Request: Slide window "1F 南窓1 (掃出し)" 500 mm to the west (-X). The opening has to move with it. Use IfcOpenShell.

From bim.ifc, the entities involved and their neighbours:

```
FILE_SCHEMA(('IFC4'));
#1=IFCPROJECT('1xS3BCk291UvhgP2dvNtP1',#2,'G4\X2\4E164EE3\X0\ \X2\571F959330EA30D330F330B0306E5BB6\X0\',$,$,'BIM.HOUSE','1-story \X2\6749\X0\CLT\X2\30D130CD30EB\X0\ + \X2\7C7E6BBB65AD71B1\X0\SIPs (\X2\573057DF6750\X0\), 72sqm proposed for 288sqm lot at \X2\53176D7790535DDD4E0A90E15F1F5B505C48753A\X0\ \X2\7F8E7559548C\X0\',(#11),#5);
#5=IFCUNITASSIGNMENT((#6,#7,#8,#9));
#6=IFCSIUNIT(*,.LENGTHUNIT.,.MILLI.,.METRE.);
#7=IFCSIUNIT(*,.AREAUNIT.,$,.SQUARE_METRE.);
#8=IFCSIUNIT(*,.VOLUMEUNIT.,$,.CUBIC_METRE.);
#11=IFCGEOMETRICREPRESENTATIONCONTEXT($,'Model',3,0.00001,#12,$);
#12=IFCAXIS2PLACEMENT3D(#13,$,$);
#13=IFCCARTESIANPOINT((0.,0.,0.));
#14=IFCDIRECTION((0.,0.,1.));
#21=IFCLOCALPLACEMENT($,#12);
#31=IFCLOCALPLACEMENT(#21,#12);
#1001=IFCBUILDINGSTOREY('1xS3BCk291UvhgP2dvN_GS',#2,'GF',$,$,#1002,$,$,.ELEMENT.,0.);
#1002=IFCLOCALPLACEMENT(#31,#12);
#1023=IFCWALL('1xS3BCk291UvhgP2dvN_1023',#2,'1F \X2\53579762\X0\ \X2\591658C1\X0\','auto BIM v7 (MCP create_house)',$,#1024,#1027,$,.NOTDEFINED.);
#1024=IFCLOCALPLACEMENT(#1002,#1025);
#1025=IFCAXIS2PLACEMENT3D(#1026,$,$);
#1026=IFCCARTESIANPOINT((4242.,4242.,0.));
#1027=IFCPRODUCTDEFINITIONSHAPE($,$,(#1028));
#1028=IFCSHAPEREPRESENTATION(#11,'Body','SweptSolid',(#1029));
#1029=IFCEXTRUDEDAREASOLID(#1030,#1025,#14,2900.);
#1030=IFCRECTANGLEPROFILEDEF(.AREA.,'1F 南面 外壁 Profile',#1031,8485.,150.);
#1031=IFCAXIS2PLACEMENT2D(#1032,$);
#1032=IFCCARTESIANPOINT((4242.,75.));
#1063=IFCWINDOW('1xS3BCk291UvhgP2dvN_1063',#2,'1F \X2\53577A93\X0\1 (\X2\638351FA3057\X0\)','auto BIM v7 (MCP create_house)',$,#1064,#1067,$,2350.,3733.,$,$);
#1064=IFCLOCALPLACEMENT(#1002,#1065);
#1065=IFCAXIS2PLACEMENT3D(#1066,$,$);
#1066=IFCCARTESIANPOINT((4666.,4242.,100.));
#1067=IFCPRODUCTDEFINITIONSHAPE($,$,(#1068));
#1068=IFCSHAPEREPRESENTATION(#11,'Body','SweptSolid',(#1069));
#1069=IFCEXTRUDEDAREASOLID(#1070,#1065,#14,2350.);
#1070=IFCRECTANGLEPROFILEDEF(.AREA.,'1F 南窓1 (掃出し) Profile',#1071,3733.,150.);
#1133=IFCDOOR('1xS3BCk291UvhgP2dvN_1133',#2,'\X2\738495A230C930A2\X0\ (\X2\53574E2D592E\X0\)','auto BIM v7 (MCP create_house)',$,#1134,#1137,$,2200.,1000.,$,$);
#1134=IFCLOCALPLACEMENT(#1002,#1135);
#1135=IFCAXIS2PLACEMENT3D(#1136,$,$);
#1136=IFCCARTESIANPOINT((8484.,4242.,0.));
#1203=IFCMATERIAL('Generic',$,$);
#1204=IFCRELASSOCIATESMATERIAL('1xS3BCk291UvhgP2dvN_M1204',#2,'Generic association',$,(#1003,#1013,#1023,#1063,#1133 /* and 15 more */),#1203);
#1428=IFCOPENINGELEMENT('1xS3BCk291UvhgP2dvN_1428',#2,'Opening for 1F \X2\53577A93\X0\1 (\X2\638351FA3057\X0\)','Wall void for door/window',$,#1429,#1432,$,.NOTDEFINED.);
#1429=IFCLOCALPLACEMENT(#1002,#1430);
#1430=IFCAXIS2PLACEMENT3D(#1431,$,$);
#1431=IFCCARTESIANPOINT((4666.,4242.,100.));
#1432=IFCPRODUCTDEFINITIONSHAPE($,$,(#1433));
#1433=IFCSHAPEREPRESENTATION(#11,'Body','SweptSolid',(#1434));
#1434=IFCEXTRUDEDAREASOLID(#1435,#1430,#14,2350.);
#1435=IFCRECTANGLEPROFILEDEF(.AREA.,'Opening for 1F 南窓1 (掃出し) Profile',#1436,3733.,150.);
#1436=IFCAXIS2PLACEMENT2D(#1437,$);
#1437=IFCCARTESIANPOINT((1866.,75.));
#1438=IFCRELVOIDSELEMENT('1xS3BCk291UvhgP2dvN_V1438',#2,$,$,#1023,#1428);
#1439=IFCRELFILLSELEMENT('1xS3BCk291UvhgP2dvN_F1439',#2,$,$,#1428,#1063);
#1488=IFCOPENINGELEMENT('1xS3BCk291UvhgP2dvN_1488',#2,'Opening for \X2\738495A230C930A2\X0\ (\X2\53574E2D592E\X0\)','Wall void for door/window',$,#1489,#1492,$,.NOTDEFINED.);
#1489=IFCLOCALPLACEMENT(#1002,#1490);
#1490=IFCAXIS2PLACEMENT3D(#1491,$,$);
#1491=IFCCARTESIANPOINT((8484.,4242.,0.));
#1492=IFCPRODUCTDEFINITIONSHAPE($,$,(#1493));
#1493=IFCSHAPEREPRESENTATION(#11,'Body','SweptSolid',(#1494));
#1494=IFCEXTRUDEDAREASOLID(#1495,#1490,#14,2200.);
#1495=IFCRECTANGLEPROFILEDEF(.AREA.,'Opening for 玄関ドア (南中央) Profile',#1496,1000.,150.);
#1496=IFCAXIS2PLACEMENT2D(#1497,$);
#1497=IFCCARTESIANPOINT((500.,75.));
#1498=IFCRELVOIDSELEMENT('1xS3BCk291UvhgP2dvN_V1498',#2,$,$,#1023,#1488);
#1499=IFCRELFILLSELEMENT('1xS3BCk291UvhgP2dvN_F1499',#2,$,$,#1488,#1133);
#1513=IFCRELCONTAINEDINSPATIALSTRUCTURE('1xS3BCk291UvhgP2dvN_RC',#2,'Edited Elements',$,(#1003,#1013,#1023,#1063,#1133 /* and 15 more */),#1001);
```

```python
import ifcopenshell
import ifcopenshell.api.geometry
import ifcopenshell.util.placement
import ifcopenshell.util.unit

model = ifcopenshell.open("bim.ifc")
unit_scale = ifcopenshell.util.unit.calculate_unit_scale(model)

window = model.by_guid("1xS3BCk291UvhgP2dvN_1063")
opening = window.FillsVoids[0].RelatingOpeningElement
wall = opening.VoidsElements[0].RelatingBuildingElement

wall_matrix = ifcopenshell.util.placement.get_local_placement(wall.ObjectPlacement)
shift = wall_matrix[:3, 0] * -0.5 / unit_scale
before = ifcopenshell.util.placement.get_local_placement(window.ObjectPlacement)[:3, 3].copy()

# The window is not placed relative to its opening, so move both.
for product in (opening, window):
    matrix = ifcopenshell.util.placement.get_local_placement(product.ObjectPlacement)
    matrix[:3, 3] += shift
    ifcopenshell.api.geometry.edit_object_placement(model, product=product, matrix=matrix, is_si=False)

after = ifcopenshell.util.placement.get_local_placement(window.ObjectPlacement)[:3, 3]
print("window moved by", (after - before).round(3) + 0.0)

model.write("bim_rev.ifc")
```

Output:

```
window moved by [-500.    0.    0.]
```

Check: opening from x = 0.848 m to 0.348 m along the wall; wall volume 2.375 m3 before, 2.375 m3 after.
